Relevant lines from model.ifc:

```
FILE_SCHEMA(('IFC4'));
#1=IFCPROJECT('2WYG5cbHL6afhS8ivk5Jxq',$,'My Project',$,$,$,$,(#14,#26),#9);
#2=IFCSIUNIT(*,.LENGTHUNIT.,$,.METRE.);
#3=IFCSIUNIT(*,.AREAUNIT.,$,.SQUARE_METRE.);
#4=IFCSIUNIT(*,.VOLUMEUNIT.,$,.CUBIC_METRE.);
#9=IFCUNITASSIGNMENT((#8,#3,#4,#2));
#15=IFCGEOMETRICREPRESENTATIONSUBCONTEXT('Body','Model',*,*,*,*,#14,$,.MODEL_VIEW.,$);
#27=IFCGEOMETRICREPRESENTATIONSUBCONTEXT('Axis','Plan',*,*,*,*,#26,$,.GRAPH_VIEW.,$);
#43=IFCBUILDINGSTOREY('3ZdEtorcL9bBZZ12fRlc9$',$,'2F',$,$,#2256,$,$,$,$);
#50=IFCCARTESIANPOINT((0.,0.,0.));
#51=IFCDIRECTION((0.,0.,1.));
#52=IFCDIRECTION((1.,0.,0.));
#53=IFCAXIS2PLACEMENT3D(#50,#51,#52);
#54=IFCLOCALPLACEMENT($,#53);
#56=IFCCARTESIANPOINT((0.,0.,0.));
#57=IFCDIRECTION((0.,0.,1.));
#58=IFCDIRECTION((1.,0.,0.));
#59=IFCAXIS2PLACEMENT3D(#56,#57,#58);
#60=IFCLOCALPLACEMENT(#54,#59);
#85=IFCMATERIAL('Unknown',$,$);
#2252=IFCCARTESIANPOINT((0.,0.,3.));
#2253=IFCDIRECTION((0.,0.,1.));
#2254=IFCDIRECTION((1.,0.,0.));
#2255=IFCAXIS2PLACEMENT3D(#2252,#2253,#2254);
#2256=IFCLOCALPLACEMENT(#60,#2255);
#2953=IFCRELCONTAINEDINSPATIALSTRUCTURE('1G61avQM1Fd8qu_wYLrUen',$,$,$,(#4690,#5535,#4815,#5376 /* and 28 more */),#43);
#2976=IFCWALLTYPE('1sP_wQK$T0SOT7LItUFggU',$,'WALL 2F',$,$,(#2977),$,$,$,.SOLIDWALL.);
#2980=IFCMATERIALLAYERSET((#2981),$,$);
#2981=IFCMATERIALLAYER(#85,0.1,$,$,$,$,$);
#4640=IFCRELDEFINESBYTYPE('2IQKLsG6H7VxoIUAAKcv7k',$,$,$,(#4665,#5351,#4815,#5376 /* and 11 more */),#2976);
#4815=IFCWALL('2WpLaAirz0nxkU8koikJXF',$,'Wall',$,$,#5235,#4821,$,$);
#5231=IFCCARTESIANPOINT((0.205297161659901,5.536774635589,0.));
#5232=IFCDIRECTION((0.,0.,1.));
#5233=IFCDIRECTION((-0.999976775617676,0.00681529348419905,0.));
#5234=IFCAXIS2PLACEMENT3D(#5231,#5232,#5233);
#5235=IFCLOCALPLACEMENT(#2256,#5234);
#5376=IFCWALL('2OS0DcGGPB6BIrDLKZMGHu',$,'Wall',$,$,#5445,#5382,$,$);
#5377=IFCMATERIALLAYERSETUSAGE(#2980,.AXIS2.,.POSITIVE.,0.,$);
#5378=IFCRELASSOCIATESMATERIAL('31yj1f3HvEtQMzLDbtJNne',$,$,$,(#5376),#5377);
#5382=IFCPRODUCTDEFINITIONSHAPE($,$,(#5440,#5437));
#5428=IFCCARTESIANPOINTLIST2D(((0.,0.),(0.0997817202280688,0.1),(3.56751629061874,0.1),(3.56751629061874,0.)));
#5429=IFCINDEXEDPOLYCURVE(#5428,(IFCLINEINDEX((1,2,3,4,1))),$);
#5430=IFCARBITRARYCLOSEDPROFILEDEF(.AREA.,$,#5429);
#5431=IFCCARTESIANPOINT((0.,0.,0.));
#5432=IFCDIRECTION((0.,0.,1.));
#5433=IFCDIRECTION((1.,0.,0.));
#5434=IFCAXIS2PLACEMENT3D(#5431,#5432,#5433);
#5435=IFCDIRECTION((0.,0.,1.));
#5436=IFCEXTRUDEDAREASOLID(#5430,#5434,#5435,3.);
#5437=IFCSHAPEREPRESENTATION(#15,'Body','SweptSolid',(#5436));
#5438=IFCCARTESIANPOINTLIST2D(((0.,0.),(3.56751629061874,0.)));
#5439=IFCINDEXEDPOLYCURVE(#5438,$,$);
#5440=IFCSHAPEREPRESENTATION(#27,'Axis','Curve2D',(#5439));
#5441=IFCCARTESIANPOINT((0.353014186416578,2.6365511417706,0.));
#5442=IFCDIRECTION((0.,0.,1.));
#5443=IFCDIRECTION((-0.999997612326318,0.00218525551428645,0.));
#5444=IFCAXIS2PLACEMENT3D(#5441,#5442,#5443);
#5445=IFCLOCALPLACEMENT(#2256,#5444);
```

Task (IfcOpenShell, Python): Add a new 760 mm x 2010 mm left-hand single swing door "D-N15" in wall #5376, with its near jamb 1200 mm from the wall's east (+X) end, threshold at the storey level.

```python
import numpy as np
import ifcopenshell
import ifcopenshell.api.feature
import ifcopenshell.api.geometry
import ifcopenshell.api.root
import ifcopenshell.api.spatial
import ifcopenshell.geom
import ifcopenshell.util.element
import ifcopenshell.util.placement
import ifcopenshell.util.representation
import ifcopenshell.util.shape
import ifcopenshell.util.unit

model = ifcopenshell.open("model.ifc")
unit_scale = ifcopenshell.util.unit.calculate_unit_scale(model)
settings = ifcopenshell.geom.settings()


def volume(element):
    """Net volume in cubic metres, openings subtracted."""
    shape = ifcopenshell.geom.create_shape(settings, element)
    return ifcopenshell.util.shape.get_volume(shape.geometry)


wall = model.by_id(5376)
storey = ifcopenshell.util.element.get_container(wall, ifc_class="IfcBuildingStorey")
context = ifcopenshell.util.representation.get_context(model, "Model", "Body", "MODEL_VIEW")
before = volume(wall)

width, height, from_end, sill = 0.76, 2.01, 1.2, 0.0  # metres

# The wall runs along its own X axis, and the end named is its -X end.
wall_shape = ifcopenshell.geom.create_shape(settings, wall)
x, y, z = ifcopenshell.util.shape.get_vertices(wall_shape.geometry).T
start = x.min() + from_end
face, thickness = float(y.min()), float(y.max() - y.min())
wall_matrix = ifcopenshell.util.placement.get_local_placement(wall.ObjectPlacement)
level = ifcopenshell.util.placement.get_local_placement(storey.ObjectPlacement)[2, 3]


def in_wall(x, y):
    """Placement at x, y metres in the wall's axes, at sill height."""
    matrix = wall_matrix.copy()
    matrix[:, 3] = wall_matrix @ np.array([x / unit_scale, y / unit_scale, 0.0, 1.0])
    matrix[2, 3] = level + sill / unit_scale
    return matrix


# Opening: a box that overshoots both wall faces by 50 mm.
opening = ifcopenshell.api.root.create_entity(model, ifc_class="IfcOpeningElement", predefined_type="OPENING")
box = ifcopenshell.api.geometry.add_wall_representation(
    model, context=context, length=width, height=height, thickness=thickness + 0.1
)
ifcopenshell.api.geometry.assign_representation(model, product=opening, representation=box)
ifcopenshell.api.geometry.edit_object_placement(model, product=opening, matrix=in_wall(start, face - 0.05), is_si=False)
ifcopenshell.api.feature.add_feature(model, feature=opening, element=wall)

door = ifcopenshell.api.root.create_entity(model, ifc_class="IfcDoor", name="D-N15", predefined_type="DOOR")
door.OverallWidth, door.OverallHeight = width / unit_scale, height / unit_scale
door.OperationType = "SINGLE_SWING_LEFT"
body = ifcopenshell.api.geometry.add_door_representation(
    model,
    context=context,
    overall_width=door.OverallWidth,
    overall_height=door.OverallHeight,
    operation_type="SINGLE_SWING_LEFT",
    lining_properties={"LiningDepth": thickness / unit_scale, "ThresholdDepth": thickness / unit_scale},
)
ifcopenshell.api.geometry.assign_representation(model, product=door, representation=body)
ifcopenshell.api.spatial.assign_container(model, products=[door], relating_structure=storey)
ifcopenshell.api.feature.add_filling(model, opening=opening, element=door)

# The lining spans the wall, so the door starts at the wall face.
ifcopenshell.api.geometry.edit_object_placement(model, product=door, matrix=in_wall(start, face), is_si=False)

after = volume(wall)

print(f"wall volume {before:.3f} -> {after:.3f} m3")

model.write("model_rev.ifc")
```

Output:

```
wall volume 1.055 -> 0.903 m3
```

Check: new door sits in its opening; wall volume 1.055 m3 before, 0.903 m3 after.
